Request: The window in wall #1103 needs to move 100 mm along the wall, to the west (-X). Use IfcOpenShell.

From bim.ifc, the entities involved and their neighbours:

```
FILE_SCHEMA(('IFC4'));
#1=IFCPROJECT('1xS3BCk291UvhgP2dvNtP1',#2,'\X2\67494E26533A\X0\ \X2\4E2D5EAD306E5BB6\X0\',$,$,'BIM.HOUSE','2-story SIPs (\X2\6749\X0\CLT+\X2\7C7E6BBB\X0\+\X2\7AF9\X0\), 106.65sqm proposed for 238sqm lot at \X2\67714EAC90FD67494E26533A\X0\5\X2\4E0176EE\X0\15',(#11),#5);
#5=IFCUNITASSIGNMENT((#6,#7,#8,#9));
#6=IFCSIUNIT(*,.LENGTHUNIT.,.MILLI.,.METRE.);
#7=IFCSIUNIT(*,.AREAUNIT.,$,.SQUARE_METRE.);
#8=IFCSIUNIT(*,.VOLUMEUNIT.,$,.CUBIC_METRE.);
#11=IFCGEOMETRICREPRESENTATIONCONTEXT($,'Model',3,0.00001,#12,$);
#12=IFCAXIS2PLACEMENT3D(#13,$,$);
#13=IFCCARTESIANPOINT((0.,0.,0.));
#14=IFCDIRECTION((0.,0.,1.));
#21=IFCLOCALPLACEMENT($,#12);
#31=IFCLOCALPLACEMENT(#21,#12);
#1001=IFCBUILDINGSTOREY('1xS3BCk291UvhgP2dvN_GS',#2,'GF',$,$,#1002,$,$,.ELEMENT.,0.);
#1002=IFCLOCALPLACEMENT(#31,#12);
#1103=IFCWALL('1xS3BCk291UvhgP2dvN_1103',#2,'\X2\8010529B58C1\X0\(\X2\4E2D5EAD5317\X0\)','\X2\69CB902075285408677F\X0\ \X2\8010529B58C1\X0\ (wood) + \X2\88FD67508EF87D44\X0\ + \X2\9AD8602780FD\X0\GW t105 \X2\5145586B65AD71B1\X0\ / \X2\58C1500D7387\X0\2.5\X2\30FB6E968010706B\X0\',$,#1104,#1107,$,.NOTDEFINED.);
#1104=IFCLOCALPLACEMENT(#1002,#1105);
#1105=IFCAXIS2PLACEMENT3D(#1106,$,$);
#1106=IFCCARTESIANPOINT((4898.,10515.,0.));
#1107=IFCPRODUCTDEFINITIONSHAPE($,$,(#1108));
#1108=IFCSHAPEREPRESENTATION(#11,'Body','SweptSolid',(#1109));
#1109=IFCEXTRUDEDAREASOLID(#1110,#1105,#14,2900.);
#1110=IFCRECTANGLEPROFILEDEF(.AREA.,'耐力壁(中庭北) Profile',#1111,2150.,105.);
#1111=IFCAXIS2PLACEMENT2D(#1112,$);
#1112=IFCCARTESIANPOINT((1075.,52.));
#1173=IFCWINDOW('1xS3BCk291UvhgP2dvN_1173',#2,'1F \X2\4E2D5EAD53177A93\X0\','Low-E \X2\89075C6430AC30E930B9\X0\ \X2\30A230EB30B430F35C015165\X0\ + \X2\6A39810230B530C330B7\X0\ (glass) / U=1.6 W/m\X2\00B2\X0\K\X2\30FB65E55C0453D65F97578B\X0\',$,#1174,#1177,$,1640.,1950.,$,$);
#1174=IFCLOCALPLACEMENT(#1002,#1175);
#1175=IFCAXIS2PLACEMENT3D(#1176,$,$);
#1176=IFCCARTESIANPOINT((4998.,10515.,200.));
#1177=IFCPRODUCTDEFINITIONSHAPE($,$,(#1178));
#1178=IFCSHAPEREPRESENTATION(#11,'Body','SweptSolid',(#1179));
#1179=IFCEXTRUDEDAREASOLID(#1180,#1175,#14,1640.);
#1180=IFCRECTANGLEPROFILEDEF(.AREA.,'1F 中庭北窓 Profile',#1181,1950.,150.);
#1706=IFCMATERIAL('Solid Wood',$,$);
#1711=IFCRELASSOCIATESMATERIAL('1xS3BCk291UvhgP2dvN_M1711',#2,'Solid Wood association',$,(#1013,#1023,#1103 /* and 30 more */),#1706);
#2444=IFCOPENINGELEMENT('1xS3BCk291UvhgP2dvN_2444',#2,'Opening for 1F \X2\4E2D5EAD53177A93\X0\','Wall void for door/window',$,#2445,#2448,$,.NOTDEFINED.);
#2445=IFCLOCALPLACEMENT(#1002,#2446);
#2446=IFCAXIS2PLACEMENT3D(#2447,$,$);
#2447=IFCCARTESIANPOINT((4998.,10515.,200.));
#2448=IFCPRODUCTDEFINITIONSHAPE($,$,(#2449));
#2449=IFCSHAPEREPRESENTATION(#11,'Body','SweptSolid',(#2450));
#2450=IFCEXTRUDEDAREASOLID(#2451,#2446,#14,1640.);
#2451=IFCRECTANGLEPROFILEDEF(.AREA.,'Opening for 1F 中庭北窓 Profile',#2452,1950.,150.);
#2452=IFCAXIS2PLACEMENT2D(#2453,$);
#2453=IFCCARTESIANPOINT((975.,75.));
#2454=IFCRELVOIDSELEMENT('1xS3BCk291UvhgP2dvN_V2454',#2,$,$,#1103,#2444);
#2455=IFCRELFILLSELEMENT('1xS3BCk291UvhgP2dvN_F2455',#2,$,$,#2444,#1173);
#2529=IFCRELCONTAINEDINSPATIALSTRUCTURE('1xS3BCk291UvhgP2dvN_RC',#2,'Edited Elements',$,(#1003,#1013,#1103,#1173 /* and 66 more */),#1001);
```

```python
import ifcopenshell
import ifcopenshell.api.geometry
import ifcopenshell.util.placement
import ifcopenshell.util.unit

model = ifcopenshell.open("bim.ifc")
unit_scale = ifcopenshell.util.unit.calculate_unit_scale(model)

window = model.by_guid("1xS3BCk291UvhgP2dvN_1173")
opening = window.FillsVoids[0].RelatingOpeningElement
wall = opening.VoidsElements[0].RelatingBuildingElement

wall_matrix = ifcopenshell.util.placement.get_local_placement(wall.ObjectPlacement)
shift = wall_matrix[:3, 0] * -0.1 / unit_scale
before = ifcopenshell.util.placement.get_local_placement(window.ObjectPlacement)[:3, 3].copy()

# The window is not placed relative to its opening, so move both.
for product in (opening, window):
    matrix = ifcopenshell.util.placement.get_local_placement(product.ObjectPlacement)
    matrix[:3, 3] += shift
    ifcopenshell.api.geometry.edit_object_placement(model, product=product, matrix=matrix, is_si=False)

after = ifcopenshell.util.placement.get_local_placement(window.ObjectPlacement)[:3, 3]
print("window moved by", (after - before).round(3) + 0.0)

model.write("bim-out.ifc")
```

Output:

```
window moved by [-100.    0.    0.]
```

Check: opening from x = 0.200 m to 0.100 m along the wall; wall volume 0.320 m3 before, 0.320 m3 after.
